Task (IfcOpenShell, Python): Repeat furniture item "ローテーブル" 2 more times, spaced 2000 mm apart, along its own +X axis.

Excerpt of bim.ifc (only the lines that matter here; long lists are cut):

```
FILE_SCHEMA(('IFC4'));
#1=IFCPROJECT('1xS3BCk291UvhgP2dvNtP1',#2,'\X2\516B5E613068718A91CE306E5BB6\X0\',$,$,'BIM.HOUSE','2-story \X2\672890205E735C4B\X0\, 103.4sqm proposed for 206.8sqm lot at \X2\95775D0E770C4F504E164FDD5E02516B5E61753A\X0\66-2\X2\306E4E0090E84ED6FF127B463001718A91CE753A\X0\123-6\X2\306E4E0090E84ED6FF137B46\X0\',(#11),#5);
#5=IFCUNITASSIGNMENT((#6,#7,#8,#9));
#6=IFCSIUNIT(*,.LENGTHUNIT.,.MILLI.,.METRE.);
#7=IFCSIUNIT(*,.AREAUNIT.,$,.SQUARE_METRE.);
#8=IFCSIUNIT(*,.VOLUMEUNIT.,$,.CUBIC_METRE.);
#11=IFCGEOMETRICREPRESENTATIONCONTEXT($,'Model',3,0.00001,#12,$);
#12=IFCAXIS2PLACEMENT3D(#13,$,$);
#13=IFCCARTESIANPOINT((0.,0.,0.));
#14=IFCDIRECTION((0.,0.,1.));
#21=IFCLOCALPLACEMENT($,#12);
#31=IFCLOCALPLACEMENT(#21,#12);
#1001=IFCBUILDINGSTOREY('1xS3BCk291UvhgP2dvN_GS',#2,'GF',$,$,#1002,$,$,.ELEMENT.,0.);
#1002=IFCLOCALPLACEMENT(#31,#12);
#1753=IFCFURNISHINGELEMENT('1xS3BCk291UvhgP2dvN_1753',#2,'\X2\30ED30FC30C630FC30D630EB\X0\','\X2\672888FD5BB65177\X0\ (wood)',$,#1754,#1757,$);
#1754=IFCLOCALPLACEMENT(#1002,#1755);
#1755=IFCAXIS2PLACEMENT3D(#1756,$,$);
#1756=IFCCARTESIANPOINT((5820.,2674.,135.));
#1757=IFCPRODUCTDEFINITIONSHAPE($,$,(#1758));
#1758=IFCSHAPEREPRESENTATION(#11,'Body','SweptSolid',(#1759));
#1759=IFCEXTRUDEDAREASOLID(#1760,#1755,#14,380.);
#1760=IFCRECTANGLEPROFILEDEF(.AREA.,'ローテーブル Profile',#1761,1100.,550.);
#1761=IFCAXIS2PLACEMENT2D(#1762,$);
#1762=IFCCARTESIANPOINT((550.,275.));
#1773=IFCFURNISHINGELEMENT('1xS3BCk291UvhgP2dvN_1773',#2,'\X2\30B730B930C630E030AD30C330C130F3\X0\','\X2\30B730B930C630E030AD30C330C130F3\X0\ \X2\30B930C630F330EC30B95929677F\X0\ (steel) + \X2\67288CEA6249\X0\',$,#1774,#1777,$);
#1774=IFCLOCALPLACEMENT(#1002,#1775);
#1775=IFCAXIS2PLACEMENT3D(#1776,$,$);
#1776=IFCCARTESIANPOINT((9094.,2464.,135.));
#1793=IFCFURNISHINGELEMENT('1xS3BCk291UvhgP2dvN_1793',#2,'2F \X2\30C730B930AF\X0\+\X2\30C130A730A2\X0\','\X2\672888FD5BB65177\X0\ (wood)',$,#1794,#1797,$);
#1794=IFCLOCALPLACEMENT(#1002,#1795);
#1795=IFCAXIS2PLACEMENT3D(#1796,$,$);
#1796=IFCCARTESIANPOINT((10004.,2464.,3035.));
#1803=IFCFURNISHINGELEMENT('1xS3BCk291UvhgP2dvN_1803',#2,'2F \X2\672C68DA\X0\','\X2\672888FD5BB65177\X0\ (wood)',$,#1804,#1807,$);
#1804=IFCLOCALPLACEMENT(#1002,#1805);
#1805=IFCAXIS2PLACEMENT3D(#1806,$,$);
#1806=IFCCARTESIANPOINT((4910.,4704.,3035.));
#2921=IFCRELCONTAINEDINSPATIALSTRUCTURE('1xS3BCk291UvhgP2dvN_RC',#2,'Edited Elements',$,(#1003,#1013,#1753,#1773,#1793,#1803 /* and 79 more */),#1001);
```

```python
import ifcopenshell
import ifcopenshell.api.geometry
import ifcopenshell.api.root
import ifcopenshell.util.element
import ifcopenshell.util.placement
import ifcopenshell.util.unit

model = ifcopenshell.open("bim.ifc")
unit_scale = ifcopenshell.util.unit.calculate_unit_scale(model)


def reuse_history(source, copy):
    """copy_class also copies each property set's owner history, people and application; keep the originals."""
    for rel in copy.IsDefinedBy:
        if rel.is_a("IfcRelDefinesByProperties") and (history := rel.RelatingPropertyDefinition.OwnerHistory):
            rel.RelatingPropertyDefinition.OwnerHistory = source.OwnerHistory
            ifcopenshell.util.element.remove_deep2(model, history)


source = model.by_guid("1xS3BCk291UvhgP2dvN_1753")
base = ifcopenshell.util.placement.get_local_placement(source.ObjectPlacement)
step = base[:3, 0] * 2 / unit_scale

for i in range(1, 3):
    copy = ifcopenshell.api.root.copy_class(model, product=source)
    copy.Representation = ifcopenshell.util.element.copy_deep(
        model, source.Representation, exclude=["IfcGeometricRepresentationContext", "IfcRepresentationMap"]
    )
    reuse_history(source, copy)
    matrix = base.copy()
    matrix[:3, 3] += i * step
    print("added at", matrix[:3, 3].round(3) + 0.0)
    ifcopenshell.api.geometry.edit_object_placement(model, product=copy, matrix=matrix, is_si=False)

model.write("bim_v2.ifc")
```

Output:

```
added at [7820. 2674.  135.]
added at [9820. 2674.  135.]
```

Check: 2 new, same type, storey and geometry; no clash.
